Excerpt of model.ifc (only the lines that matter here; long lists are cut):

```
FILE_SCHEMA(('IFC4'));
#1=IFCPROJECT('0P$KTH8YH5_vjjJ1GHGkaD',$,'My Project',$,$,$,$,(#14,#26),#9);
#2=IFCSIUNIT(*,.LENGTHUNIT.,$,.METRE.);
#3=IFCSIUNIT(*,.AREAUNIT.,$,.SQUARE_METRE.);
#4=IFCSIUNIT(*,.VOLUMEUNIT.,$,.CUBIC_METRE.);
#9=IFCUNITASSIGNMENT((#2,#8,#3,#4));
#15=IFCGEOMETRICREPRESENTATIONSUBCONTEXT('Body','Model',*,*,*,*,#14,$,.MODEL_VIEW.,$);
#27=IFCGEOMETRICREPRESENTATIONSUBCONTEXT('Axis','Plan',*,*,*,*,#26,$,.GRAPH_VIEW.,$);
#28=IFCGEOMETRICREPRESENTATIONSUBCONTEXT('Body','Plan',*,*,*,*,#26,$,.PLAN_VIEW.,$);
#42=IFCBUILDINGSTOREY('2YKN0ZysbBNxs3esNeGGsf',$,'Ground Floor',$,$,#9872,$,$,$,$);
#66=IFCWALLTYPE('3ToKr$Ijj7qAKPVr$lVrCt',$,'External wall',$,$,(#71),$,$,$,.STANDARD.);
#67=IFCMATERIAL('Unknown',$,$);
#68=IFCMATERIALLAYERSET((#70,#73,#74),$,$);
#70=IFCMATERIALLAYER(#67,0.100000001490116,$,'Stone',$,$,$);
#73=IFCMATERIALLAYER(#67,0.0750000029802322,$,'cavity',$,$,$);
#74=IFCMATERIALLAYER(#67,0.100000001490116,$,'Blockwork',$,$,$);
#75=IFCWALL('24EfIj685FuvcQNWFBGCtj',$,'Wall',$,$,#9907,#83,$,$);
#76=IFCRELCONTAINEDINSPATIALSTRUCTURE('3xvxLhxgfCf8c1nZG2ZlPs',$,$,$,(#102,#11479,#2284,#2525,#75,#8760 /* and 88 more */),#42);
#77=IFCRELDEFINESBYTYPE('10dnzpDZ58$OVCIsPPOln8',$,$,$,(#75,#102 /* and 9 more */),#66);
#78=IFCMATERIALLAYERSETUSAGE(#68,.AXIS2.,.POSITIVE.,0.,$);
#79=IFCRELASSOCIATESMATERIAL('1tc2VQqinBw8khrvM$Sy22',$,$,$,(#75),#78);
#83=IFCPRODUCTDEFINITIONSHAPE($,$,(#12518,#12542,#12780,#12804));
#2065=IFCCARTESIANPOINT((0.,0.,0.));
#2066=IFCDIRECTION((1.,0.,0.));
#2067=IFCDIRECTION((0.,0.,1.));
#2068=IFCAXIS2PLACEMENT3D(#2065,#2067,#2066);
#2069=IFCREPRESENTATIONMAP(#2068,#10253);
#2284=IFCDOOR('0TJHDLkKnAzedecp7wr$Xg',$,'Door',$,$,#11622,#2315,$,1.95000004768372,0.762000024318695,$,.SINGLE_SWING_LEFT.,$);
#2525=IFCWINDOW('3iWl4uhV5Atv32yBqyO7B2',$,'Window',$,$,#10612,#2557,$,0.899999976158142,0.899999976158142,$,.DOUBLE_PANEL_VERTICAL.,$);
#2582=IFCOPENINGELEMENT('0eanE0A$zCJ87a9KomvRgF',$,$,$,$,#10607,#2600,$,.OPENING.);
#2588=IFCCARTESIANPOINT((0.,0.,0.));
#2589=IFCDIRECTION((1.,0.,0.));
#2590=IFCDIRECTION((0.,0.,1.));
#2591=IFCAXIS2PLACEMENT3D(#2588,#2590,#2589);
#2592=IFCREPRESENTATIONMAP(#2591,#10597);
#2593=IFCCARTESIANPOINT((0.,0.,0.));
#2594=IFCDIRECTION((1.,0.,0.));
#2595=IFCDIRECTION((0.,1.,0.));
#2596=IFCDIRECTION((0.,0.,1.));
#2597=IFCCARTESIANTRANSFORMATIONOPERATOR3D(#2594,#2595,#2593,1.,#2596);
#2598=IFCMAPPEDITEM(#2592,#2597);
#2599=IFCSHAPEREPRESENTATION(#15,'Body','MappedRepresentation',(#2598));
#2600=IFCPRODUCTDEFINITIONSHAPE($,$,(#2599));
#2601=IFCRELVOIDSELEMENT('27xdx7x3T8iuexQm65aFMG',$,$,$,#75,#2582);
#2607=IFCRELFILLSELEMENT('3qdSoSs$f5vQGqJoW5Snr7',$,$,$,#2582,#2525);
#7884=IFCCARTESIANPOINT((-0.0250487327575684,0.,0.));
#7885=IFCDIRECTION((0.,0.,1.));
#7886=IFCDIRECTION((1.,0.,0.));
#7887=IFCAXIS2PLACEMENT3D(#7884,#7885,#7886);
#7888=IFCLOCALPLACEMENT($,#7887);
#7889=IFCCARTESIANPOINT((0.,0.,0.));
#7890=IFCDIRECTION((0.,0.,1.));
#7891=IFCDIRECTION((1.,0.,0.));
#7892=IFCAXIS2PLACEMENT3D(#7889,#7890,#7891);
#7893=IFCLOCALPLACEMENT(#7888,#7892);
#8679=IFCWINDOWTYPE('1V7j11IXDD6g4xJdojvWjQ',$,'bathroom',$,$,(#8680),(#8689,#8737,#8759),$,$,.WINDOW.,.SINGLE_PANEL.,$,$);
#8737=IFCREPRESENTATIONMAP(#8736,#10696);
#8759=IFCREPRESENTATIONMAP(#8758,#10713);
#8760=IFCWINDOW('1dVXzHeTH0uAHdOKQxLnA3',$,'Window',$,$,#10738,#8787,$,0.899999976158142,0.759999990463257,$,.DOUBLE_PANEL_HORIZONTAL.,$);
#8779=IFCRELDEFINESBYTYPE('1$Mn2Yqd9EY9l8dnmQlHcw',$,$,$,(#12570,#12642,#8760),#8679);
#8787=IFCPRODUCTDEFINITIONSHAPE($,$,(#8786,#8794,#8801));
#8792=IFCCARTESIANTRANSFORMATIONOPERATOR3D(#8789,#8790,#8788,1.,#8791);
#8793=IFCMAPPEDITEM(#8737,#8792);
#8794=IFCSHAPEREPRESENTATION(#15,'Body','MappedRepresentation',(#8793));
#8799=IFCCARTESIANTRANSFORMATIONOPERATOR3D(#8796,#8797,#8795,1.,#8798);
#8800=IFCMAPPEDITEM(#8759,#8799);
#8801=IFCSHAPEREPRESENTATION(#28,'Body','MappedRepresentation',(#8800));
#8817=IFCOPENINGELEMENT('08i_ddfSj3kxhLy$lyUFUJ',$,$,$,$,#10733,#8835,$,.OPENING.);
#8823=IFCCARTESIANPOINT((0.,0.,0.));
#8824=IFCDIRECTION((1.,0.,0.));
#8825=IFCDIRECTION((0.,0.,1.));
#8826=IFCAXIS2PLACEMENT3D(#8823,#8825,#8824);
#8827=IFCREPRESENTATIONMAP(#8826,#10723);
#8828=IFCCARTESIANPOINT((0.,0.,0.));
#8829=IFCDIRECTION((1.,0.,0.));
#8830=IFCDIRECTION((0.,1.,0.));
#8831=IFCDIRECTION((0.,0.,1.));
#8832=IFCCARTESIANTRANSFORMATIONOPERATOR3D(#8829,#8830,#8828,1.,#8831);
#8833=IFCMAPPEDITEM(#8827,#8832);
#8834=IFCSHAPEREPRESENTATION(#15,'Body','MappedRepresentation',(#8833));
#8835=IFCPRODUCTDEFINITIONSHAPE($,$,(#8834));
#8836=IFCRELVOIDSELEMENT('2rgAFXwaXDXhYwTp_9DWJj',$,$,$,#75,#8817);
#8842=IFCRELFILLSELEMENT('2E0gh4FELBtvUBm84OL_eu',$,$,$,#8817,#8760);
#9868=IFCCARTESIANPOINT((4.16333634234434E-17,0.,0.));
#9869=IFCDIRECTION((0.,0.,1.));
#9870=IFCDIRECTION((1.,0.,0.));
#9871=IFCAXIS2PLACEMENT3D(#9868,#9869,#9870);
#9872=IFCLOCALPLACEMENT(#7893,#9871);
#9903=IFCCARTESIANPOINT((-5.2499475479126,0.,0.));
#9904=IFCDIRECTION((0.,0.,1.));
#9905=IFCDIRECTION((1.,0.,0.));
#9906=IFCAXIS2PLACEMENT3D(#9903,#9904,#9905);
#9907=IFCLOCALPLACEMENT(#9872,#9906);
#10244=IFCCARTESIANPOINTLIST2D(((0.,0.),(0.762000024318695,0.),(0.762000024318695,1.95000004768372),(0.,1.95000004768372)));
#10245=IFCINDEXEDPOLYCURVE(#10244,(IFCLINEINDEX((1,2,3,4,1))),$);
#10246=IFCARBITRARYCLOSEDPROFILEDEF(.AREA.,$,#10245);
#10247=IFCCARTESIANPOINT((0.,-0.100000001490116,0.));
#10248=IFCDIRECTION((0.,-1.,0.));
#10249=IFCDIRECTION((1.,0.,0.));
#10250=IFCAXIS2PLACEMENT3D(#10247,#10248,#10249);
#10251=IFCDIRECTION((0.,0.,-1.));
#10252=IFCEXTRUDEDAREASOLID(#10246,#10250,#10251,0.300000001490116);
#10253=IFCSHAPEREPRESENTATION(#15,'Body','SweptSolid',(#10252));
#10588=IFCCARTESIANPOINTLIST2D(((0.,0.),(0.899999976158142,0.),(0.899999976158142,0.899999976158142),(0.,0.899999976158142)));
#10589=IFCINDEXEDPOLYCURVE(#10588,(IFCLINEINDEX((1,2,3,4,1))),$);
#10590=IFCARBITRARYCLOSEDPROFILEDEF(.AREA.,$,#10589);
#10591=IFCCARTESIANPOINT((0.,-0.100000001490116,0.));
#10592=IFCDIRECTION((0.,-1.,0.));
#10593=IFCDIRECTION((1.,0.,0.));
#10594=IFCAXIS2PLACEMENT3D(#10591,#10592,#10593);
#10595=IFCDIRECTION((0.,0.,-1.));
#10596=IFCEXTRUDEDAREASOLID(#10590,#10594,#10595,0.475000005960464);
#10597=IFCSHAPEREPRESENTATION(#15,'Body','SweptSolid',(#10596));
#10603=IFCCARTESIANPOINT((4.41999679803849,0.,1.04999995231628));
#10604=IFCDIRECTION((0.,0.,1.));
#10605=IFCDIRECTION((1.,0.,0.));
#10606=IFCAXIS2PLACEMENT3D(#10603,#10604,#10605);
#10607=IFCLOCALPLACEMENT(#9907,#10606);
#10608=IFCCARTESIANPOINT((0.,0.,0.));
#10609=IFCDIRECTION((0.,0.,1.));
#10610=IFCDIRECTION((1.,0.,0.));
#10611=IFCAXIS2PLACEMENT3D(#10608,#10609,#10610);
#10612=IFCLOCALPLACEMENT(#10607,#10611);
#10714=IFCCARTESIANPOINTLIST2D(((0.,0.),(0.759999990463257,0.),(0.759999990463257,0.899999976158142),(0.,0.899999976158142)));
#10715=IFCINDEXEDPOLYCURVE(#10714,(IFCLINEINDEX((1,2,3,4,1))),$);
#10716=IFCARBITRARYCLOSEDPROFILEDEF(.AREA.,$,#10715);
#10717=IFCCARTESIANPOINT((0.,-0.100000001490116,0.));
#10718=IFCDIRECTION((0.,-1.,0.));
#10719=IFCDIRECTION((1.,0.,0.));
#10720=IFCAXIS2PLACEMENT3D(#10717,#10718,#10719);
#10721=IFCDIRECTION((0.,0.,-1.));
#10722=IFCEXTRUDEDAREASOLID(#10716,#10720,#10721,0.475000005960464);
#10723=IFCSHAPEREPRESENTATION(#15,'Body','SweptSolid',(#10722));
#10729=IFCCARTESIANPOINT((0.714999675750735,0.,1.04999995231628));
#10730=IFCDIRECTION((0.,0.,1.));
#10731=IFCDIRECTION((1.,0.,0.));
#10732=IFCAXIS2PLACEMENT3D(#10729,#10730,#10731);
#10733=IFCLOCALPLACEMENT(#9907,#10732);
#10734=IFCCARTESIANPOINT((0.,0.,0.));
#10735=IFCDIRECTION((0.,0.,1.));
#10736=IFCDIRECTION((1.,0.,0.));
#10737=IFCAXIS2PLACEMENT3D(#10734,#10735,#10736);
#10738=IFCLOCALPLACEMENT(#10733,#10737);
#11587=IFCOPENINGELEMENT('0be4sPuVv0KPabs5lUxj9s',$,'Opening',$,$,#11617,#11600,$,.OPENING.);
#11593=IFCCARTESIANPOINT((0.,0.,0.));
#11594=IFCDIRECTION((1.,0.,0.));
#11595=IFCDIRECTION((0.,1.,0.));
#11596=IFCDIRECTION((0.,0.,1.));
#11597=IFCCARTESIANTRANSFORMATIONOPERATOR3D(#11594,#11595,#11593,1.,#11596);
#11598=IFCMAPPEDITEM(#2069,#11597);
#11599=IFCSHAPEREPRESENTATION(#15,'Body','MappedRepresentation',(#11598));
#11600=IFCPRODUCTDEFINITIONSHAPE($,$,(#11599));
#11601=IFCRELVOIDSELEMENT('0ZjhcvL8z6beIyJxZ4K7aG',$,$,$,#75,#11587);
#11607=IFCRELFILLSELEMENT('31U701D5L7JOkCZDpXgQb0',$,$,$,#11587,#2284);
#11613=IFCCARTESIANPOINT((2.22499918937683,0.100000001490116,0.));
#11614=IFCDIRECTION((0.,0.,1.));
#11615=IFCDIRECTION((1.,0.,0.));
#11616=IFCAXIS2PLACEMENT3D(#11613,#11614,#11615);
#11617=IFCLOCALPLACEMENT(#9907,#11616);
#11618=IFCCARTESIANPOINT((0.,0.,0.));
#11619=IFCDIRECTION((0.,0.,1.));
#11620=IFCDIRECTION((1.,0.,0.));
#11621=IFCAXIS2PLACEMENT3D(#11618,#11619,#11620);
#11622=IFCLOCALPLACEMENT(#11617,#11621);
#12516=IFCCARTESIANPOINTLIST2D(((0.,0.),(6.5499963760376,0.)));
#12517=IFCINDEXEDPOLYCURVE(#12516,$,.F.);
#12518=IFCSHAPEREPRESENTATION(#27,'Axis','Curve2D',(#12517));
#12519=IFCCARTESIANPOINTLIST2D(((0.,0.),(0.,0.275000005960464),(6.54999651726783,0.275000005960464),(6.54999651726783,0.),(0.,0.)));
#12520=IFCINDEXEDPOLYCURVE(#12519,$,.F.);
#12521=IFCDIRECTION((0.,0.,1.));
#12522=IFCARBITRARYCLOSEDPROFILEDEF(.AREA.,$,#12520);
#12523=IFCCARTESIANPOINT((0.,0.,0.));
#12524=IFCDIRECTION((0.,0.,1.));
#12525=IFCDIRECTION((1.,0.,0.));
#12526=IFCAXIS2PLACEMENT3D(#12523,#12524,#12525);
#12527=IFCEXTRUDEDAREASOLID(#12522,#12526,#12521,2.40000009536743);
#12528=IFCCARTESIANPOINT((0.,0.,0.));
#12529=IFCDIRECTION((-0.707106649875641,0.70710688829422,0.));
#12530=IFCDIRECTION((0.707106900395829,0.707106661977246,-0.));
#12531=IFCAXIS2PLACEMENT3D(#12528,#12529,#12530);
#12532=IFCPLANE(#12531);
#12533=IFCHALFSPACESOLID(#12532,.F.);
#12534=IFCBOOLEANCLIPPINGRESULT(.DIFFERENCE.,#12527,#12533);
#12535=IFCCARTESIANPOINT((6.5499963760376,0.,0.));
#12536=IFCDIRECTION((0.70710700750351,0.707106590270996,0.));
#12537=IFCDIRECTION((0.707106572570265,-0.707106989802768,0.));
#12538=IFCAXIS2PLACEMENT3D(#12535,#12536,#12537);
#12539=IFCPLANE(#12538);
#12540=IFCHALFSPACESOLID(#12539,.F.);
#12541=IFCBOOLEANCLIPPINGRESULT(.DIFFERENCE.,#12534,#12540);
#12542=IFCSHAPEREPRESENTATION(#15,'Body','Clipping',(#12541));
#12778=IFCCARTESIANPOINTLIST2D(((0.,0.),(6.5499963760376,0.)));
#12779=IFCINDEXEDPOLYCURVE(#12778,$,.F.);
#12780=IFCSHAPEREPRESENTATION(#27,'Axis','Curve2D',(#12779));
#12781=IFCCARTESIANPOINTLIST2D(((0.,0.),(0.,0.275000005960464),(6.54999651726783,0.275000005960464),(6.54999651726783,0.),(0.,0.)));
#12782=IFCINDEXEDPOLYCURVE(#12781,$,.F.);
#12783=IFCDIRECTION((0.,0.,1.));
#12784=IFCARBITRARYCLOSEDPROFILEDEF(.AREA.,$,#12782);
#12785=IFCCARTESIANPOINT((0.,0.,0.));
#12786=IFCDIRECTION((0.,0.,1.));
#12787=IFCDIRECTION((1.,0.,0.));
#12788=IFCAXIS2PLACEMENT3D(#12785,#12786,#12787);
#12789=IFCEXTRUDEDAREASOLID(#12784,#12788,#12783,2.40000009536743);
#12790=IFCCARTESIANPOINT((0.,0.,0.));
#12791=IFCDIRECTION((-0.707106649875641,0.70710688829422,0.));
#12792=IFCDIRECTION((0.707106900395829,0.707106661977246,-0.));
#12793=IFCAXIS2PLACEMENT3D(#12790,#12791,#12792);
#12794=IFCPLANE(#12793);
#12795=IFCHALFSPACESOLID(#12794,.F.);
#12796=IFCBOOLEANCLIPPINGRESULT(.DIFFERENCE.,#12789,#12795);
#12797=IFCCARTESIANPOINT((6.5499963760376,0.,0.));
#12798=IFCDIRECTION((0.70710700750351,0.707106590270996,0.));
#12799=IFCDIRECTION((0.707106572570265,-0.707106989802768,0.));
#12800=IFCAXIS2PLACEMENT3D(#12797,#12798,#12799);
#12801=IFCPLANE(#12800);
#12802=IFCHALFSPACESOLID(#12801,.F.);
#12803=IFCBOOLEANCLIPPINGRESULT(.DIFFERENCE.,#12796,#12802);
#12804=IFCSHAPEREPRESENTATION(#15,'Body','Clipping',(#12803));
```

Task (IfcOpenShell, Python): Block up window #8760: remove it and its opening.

```python
import ifcopenshell
import ifcopenshell.api.feature
import ifcopenshell.api.root
import ifcopenshell.geom
import ifcopenshell.util.shape

model = ifcopenshell.open("model.ifc")
settings = ifcopenshell.geom.settings()


def volume(element):
    """Net volume in cubic metres, openings subtracted."""
    shape = ifcopenshell.geom.create_shape(settings, element)
    return ifcopenshell.util.shape.get_volume(shape.geometry)


window = model.by_guid("1dVXzHeTH0uAHdOKQxLnA3")
opening = window.FillsVoids[0].RelatingOpeningElement
wall = opening.VoidsElements[0].RelatingBuildingElement
before = volume(wall)

ifcopenshell.api.root.remove_product(model, product=window)
ifcopenshell.api.feature.remove_feature(model, feature=opening)

after = volume(wall)

print(f"wall volume {before:.3f} -> {after:.3f} m3")

model.write("model_rev.ifc")
```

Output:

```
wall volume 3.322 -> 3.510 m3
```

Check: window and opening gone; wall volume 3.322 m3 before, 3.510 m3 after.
